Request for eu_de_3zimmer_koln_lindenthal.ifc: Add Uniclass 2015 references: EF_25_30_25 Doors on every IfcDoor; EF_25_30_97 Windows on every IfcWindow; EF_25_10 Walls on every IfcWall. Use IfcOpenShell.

First a look at what the model holds.

```python
import ifcopenshell

model = ifcopenshell.open("eu_de_3zimmer_koln_lindenthal.ifc")
print(model.schema)
print("classifications:", [c.Name for c in model.by_type("IfcClassification")])
for ifc_class in ("IfcDoor", "IfcRoof", "IfcStair", "IfcWall", "IfcWindow"):
    print(ifc_class, len(model.by_type(ifc_class)))
```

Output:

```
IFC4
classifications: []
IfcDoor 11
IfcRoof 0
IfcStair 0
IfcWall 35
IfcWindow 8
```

```python
import ifcopenshell
import ifcopenshell.api.classification

model = ifcopenshell.open("eu_de_3zimmer_koln_lindenthal.ifc")

system = ifcopenshell.api.classification.add_classification(model, classification="Uniclass 2015")

codes = {
    "IfcDoor": ("EF_25_30_25", "Doors"),
    "IfcWindow": ("EF_25_30_97", "Windows"),
    "IfcWall": ("EF_25_10", "Walls"),
}
for ifc_class, (code, name) in codes.items():
    products = model.by_type(ifc_class)
    ifcopenshell.api.classification.add_reference(
        model, products=products, classification=system, identification=code, name=name
    )
    print(code, len(products))

model.write("eu_de_3zimmer_koln_lindenthal_updated.ifc")
```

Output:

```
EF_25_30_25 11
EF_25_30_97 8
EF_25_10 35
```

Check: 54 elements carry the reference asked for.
